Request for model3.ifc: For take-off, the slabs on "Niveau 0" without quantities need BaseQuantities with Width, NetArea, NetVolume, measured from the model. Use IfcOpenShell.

First a look at what the model holds.

```python
import ifcopenshell
import ifcopenshell.util.element
import ifcopenshell.util.unit

model = ifcopenshell.open("model3.ifc")
print(model.schema)
for unit_type in ("LENGTHUNIT", "AREAUNIT", "VOLUMEUNIT"):
    print(unit_type, ifcopenshell.util.unit.calculate_unit_scale(model, unit_type))
storey = next(s for s in model.by_type("IfcBuildingStorey") if s.Name == "Niveau 0")
slabs = [e for e in ifcopenshell.util.element.get_decomposition(storey) if e.is_a("IfcSlab")]
for e in sorted(slabs, key=lambda e: e.id()):
    print(e.id(), e.is_a(), e.Name, list(ifcopenshell.util.element.get_psets(e, qtos_only=True)), sep=" | ")
```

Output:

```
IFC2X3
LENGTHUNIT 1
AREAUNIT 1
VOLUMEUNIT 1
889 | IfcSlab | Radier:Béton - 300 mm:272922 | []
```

```python
import ifcopenshell
import ifcopenshell.api.pset
import ifcopenshell.geom
import ifcopenshell.util.element
import ifcopenshell.util.shape
import ifcopenshell.util.unit

model = ifcopenshell.open("model3.ifc")
unit_scale = ifcopenshell.util.unit.calculate_unit_scale(model)
area_scale = ifcopenshell.util.unit.calculate_unit_scale(model, "AREAUNIT")
volume_scale = ifcopenshell.util.unit.calculate_unit_scale(model, "VOLUMEUNIT")
settings = ifcopenshell.geom.settings()

storey = next(s for s in model.by_type("IfcBuildingStorey") if s.Name == "Niveau 0")
slabs = [e for e in ifcopenshell.util.element.get_decomposition(storey) if e.is_a("IfcSlab")]

for e in sorted(slabs, key=lambda e: e.id()):
    if ifcopenshell.util.element.get_psets(e, qtos_only=True, should_inherit=False):
        continue
    # Geometry comes back in metres, in the element's own axes.
    shape = ifcopenshell.geom.create_shape(settings, e)
    values = {
        "Width": ifcopenshell.util.shape.get_z(shape.geometry) / unit_scale,
        "NetArea": ifcopenshell.util.shape.get_footprint_area(shape.geometry) / area_scale,
        "NetVolume": ifcopenshell.util.shape.get_volume(shape.geometry) / volume_scale,
    }
    qto = ifcopenshell.api.pset.add_qto(model, product=e, name="BaseQuantities")
    ifcopenshell.api.pset.edit_qto(model, qto=qto, properties=values)
    print(e.id(), {k: round(v, 3) for k, v in values.items()})

model.write("model3_edited.ifc")
```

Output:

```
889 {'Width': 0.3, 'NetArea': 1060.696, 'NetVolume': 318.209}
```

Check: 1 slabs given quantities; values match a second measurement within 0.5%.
